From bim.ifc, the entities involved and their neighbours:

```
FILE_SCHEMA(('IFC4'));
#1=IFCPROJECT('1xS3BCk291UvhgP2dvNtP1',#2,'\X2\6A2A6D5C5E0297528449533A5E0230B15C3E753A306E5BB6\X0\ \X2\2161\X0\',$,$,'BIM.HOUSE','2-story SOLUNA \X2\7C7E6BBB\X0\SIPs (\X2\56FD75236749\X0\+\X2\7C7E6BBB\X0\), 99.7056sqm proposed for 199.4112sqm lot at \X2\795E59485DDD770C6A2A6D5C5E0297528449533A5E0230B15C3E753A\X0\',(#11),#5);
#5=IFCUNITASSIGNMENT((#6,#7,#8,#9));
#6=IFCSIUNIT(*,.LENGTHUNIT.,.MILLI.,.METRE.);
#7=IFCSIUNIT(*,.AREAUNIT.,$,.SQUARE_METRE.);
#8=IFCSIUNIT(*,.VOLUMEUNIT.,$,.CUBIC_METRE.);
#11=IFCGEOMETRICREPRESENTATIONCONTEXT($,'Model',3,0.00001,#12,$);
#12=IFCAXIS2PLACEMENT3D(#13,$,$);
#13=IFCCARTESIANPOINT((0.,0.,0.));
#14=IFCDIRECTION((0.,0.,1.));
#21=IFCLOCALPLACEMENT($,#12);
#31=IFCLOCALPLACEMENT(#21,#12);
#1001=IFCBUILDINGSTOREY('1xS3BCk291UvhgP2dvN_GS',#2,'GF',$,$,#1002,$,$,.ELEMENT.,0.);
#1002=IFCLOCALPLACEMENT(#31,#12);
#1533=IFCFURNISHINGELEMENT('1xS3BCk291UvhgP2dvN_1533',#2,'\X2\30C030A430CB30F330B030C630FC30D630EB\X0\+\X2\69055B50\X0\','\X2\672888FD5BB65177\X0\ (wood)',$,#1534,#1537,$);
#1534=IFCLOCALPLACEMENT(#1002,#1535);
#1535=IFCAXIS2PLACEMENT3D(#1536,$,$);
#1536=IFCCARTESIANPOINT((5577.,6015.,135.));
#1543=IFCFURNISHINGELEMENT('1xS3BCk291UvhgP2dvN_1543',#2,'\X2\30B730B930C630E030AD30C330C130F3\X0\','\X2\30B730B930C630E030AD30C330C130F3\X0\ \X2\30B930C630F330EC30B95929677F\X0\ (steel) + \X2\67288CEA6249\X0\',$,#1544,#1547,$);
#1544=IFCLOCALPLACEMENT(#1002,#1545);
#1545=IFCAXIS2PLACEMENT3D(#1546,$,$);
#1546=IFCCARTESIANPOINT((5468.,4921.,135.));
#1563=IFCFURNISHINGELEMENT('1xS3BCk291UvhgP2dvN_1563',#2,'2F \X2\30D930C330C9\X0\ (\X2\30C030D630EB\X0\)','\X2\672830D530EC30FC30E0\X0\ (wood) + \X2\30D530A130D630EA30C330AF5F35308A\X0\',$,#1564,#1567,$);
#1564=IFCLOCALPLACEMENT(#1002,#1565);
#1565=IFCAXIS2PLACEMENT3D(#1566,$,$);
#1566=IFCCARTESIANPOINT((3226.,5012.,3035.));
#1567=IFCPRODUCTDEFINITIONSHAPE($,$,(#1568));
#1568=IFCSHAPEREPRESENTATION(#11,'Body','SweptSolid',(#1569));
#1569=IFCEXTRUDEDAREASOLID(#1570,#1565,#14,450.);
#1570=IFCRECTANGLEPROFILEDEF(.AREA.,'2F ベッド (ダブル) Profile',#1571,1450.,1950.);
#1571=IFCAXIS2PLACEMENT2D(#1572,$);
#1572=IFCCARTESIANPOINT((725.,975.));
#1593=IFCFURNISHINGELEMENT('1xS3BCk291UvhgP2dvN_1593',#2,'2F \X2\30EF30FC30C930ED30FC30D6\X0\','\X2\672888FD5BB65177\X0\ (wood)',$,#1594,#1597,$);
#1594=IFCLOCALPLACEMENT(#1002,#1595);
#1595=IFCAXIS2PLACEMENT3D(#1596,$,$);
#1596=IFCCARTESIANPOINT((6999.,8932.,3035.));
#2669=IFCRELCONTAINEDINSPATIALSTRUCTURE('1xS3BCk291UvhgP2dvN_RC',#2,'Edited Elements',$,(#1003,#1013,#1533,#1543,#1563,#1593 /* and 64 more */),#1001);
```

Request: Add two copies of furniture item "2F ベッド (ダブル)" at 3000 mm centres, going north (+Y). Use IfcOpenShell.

```python
import numpy as np
import ifcopenshell
import ifcopenshell.api.geometry
import ifcopenshell.api.root
import ifcopenshell.util.element
import ifcopenshell.util.placement
import ifcopenshell.util.unit

model = ifcopenshell.open("bim.ifc")
unit_scale = ifcopenshell.util.unit.calculate_unit_scale(model)


def reuse_history(source, copy):
    """copy_class also copies each property set's owner history, people and application; keep the originals."""
    for rel in copy.IsDefinedBy:
        if rel.is_a("IfcRelDefinesByProperties") and (history := rel.RelatingPropertyDefinition.OwnerHistory):
            rel.RelatingPropertyDefinition.OwnerHistory = source.OwnerHistory
            ifcopenshell.util.element.remove_deep2(model, history)


source = model.by_id(1563)
base = ifcopenshell.util.placement.get_local_placement(source.ObjectPlacement)
step = np.array([0.0, 1.0, 0.0]) * 3 / unit_scale

for i in range(1, 3):
    copy = ifcopenshell.api.root.copy_class(model, product=source)
    copy.Representation = ifcopenshell.util.element.copy_deep(
        model, source.Representation, exclude=["IfcGeometricRepresentationContext", "IfcRepresentationMap"]
    )
    reuse_history(source, copy)
    matrix = base.copy()
    matrix[:3, 3] += i * step
    print("added at", matrix[:3, 3].round(3) + 0.0)
    ifcopenshell.api.geometry.edit_object_placement(model, product=copy, matrix=matrix, is_si=False)

model.write("bim_v2.ifc")
```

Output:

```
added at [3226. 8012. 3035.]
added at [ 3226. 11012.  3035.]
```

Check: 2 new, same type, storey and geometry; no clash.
